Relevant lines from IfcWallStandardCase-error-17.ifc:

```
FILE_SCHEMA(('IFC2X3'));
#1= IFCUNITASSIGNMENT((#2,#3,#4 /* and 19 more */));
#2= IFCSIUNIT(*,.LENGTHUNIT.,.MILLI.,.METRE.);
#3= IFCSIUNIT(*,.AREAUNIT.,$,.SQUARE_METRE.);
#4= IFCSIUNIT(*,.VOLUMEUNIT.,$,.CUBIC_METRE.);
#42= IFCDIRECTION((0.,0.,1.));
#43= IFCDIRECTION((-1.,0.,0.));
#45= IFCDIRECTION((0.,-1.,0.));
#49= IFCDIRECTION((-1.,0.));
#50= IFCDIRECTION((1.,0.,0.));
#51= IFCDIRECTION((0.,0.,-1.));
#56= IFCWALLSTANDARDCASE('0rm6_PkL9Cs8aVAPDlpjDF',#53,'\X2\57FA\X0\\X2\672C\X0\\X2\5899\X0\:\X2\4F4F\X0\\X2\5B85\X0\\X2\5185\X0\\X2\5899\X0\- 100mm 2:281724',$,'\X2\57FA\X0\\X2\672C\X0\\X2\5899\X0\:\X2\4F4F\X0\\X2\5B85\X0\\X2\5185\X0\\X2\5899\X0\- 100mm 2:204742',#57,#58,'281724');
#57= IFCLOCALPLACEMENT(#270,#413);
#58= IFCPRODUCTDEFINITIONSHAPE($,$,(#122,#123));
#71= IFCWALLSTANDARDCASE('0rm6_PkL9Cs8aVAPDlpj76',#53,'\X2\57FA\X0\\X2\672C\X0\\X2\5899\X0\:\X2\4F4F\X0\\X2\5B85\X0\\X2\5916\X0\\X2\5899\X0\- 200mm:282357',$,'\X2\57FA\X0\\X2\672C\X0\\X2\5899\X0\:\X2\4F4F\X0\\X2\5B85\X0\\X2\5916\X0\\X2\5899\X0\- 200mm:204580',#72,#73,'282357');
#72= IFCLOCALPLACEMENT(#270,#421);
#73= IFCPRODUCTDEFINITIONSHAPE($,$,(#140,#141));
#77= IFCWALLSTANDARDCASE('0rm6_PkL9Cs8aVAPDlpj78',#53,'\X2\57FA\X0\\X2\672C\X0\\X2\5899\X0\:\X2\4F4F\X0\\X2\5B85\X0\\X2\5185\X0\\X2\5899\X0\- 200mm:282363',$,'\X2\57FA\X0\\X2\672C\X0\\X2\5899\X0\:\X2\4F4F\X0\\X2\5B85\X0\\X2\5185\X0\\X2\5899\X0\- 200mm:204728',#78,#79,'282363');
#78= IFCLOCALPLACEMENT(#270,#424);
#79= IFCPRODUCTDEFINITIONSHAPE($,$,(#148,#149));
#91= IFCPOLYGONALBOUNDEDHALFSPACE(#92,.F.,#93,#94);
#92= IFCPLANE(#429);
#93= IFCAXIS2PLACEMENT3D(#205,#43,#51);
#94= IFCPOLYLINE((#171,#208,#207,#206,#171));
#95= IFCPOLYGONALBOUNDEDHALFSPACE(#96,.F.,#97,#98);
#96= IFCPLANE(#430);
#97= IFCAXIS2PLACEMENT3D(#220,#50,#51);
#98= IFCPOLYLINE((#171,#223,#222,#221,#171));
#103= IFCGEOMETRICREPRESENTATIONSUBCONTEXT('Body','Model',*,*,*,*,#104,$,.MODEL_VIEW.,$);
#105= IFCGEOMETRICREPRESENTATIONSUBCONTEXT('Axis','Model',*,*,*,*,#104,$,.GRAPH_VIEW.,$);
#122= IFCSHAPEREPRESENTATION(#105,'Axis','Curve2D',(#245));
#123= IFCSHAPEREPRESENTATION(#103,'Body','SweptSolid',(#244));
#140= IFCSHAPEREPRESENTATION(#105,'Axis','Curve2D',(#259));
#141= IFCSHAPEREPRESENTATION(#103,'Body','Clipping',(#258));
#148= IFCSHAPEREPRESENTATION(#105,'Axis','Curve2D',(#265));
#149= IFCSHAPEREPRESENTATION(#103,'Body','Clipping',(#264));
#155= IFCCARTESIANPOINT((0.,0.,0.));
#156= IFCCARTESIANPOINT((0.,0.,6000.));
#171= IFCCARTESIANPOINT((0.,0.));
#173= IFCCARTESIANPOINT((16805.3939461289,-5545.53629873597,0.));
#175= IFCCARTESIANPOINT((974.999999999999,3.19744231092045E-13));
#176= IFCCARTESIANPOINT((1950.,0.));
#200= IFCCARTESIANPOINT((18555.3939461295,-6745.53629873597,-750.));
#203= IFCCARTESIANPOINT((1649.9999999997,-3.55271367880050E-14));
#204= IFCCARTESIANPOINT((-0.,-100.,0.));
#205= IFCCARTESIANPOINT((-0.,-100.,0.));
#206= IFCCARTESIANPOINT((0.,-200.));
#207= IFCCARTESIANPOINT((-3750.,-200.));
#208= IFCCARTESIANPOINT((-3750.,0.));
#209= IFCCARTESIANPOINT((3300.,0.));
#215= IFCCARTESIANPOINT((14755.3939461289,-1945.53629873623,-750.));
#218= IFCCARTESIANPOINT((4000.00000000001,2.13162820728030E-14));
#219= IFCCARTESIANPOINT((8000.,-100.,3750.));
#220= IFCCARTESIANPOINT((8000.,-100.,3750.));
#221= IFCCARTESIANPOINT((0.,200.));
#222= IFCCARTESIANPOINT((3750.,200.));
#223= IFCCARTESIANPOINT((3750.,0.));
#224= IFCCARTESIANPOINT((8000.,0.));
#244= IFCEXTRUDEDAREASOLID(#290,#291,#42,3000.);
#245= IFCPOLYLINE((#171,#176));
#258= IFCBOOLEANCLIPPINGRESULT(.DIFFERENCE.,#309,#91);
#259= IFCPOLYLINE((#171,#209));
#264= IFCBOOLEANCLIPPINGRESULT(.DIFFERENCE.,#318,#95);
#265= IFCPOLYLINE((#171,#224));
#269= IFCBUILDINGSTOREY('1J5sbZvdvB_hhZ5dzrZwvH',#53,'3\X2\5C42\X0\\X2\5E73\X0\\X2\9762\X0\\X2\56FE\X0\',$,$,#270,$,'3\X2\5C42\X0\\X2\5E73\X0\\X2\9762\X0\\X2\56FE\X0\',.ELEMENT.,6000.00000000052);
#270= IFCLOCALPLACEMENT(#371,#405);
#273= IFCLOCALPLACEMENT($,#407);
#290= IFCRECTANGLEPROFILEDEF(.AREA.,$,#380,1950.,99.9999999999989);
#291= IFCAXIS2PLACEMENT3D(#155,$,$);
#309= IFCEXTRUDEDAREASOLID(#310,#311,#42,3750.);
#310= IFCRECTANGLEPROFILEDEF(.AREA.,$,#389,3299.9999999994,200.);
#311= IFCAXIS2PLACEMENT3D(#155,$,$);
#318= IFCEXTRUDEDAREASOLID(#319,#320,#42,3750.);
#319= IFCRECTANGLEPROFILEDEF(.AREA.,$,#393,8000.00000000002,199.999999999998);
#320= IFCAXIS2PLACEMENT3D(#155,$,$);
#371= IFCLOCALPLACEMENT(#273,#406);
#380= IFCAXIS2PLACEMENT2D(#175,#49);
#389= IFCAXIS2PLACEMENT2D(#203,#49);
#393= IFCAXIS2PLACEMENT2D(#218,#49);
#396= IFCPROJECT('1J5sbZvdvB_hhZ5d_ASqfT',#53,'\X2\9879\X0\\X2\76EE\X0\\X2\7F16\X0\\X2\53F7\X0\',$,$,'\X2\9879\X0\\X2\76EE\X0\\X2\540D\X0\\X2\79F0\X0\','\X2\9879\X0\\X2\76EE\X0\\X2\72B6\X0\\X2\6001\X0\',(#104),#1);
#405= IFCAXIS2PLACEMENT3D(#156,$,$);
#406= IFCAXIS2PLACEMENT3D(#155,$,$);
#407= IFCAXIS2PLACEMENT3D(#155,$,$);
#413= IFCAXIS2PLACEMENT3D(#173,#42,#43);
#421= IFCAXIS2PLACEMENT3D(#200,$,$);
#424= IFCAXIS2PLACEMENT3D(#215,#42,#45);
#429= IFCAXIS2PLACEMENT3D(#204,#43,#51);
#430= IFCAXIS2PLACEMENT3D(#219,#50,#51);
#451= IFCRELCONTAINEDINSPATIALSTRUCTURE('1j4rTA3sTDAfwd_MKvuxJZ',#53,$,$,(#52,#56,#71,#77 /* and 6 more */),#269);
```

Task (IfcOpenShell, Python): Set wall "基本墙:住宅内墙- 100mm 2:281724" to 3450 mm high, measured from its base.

```python
import ifcopenshell
import ifcopenshell.geom
import ifcopenshell.util.representation
import ifcopenshell.util.shape
import ifcopenshell.util.unit

model = ifcopenshell.open("IfcWallStandardCase-error-17.ifc")
unit_scale = ifcopenshell.util.unit.calculate_unit_scale(model)
settings = ifcopenshell.geom.settings()


def volume(element):
    """Net volume in cubic metres, openings subtracted."""
    shape = ifcopenshell.geom.create_shape(settings, element)
    return ifcopenshell.util.shape.get_volume(shape.geometry)


wall = model.by_id(56)
before = volume(wall)

body = ifcopenshell.util.representation.get_representation(wall, "Model", "Body")
solid = body.Items[0]
old_height = solid.Depth
solid.Depth = 3.45 / unit_scale
after = volume(wall)

print(f"height {old_height:g} -> {solid.Depth:g}, volume {before:.3f} -> {after:.3f} m3")

model.write("IfcWallStandardCase-error-17_edited.ifc")
```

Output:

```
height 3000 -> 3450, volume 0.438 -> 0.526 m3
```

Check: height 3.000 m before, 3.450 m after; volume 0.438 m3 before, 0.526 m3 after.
